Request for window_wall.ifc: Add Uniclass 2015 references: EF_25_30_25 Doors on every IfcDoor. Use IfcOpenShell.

First a look at what the model holds.

```python
import ifcopenshell

model = ifcopenshell.open("window_wall.ifc")
print(model.schema)
print("classifications:", [c.Name for c in model.by_type("IfcClassification")])
for ifc_class in ("IfcDoor", "IfcRoof", "IfcStair", "IfcWall", "IfcWindow"):
    print(ifc_class, len(model.by_type(ifc_class)))
```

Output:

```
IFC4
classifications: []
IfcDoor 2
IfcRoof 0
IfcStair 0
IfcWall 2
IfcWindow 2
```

```python
import ifcopenshell
import ifcopenshell.api.classification

model = ifcopenshell.open("window_wall.ifc")

system = ifcopenshell.api.classification.add_classification(model, classification="Uniclass 2015")

codes = {
    "IfcDoor": ("EF_25_30_25", "Doors"),
}
for ifc_class, (code, name) in codes.items():
    products = model.by_type(ifc_class)
    ifcopenshell.api.classification.add_reference(
        model, products=products, classification=system, identification=code, name=name
    )
    print(code, len(products))

model.write("window_wall_v2.ifc")
```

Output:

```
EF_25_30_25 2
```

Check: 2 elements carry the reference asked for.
